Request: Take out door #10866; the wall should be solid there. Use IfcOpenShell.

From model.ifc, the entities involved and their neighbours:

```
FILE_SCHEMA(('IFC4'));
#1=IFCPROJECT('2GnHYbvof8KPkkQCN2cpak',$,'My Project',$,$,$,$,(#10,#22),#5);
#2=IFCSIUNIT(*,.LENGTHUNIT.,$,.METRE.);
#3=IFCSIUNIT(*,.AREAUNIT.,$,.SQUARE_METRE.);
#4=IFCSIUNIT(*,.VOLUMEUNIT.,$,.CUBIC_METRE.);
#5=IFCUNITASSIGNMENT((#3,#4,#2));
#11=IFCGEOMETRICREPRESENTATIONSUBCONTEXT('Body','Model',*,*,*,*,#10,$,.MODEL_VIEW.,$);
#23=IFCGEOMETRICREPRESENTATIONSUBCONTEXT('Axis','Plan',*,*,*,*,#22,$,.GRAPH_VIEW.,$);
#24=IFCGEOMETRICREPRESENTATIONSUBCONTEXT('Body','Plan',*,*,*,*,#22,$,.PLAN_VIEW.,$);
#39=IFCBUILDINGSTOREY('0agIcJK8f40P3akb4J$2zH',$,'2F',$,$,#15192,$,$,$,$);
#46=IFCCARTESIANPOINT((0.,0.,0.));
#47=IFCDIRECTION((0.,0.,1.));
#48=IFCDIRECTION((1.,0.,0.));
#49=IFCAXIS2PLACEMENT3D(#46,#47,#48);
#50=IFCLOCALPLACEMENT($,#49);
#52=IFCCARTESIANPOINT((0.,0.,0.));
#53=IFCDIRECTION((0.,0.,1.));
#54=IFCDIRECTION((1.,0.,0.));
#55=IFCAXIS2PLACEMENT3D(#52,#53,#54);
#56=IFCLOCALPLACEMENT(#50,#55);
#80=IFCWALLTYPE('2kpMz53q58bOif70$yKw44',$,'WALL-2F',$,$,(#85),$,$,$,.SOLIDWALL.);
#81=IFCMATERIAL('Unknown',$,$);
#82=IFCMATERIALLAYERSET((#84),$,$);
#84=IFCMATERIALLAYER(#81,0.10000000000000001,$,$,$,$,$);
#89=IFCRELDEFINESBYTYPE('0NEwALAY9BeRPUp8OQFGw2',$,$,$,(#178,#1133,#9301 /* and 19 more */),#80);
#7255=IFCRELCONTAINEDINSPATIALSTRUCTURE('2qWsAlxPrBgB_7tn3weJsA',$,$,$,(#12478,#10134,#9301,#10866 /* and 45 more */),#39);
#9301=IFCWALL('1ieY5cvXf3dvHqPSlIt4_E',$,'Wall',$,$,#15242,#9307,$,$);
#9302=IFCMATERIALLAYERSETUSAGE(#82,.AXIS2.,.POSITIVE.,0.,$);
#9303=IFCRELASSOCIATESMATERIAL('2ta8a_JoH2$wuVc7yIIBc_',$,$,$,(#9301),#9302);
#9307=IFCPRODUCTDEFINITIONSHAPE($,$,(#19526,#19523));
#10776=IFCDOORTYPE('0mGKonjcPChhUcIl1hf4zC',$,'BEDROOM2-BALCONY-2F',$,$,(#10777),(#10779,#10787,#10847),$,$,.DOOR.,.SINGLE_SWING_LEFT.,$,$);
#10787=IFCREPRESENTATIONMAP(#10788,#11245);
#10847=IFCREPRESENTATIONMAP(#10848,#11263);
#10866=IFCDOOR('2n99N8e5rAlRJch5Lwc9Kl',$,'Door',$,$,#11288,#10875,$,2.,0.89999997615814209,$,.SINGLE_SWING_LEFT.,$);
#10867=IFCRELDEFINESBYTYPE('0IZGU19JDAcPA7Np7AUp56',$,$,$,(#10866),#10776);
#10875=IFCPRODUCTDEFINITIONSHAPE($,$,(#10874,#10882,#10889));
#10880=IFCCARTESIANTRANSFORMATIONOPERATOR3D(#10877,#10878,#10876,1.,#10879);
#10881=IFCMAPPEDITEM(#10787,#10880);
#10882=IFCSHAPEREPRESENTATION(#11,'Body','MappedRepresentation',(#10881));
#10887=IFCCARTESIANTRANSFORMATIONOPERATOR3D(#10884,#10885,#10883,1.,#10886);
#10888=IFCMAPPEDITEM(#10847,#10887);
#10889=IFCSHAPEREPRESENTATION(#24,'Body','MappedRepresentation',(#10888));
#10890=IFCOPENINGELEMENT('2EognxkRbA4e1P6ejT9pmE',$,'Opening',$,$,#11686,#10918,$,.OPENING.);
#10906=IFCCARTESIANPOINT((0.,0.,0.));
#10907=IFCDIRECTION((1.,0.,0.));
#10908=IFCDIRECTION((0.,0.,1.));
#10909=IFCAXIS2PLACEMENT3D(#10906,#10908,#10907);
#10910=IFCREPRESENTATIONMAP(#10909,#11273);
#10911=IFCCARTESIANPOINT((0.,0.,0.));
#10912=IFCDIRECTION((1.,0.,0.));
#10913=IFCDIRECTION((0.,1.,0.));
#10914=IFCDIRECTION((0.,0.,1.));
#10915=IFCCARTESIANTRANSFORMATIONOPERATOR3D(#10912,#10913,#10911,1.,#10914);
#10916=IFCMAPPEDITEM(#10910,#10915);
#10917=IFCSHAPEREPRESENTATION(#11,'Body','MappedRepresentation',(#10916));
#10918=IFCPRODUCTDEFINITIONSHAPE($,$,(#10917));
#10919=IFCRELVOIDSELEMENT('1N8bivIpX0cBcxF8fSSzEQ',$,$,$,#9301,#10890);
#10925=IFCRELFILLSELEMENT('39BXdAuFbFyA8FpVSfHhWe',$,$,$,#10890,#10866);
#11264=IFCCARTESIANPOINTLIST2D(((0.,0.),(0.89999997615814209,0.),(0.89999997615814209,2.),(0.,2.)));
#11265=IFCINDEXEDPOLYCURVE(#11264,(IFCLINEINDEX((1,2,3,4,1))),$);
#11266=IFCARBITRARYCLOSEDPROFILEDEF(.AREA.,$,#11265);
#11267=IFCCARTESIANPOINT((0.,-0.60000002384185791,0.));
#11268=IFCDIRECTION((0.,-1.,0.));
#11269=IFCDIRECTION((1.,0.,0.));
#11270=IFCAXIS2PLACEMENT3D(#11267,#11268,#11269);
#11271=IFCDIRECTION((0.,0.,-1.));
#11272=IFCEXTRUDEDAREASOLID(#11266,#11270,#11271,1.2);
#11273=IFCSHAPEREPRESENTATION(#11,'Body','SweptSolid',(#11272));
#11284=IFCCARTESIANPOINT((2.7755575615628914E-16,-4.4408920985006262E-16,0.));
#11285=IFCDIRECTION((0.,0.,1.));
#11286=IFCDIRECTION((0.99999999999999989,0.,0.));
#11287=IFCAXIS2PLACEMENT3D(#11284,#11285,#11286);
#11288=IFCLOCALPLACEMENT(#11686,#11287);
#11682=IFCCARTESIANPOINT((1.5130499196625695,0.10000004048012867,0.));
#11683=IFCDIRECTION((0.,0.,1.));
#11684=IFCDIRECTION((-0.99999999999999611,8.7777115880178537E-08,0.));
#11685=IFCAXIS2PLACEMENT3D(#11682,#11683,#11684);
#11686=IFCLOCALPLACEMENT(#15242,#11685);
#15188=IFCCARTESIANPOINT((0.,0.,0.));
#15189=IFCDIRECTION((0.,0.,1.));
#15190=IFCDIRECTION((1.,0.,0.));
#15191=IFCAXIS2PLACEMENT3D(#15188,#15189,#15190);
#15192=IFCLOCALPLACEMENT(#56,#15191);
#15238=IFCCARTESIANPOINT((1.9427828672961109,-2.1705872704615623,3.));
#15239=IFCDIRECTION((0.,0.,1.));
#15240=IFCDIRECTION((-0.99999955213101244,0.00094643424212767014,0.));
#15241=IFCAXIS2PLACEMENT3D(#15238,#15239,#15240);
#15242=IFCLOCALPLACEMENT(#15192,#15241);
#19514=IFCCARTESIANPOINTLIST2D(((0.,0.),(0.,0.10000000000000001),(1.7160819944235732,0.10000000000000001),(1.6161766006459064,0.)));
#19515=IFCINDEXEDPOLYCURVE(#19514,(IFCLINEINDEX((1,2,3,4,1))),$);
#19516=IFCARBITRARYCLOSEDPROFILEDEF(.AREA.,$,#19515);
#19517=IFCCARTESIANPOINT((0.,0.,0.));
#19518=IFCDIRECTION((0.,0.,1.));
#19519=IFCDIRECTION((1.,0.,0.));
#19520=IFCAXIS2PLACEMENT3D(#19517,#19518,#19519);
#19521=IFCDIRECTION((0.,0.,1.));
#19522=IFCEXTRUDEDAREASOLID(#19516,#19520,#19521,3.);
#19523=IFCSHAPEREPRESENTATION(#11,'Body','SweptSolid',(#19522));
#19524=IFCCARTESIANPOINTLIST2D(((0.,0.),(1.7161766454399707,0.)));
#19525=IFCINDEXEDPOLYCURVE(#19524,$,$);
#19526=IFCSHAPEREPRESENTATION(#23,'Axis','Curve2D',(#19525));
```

```python
import ifcopenshell
import ifcopenshell.api.feature
import ifcopenshell.api.root
import ifcopenshell.geom
import ifcopenshell.util.shape

model = ifcopenshell.open("model.ifc")
settings = ifcopenshell.geom.settings()


def volume(element):
    """Net volume in cubic metres, openings subtracted."""
    shape = ifcopenshell.geom.create_shape(settings, element)
    return ifcopenshell.util.shape.get_volume(shape.geometry)


door = model.by_guid("2n99N8e5rAlRJch5Lwc9Kl")
opening = door.FillsVoids[0].RelatingOpeningElement
wall = opening.VoidsElements[0].RelatingBuildingElement
before = volume(wall)

ifcopenshell.api.root.remove_product(model, product=door)
ifcopenshell.api.feature.remove_feature(model, feature=opening)

after = volume(wall)

print(f"wall volume {before:.3f} -> {after:.3f} m3")

model.write("model_updated.ifc")
```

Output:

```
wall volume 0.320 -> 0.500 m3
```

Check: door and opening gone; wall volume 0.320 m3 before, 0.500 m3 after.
